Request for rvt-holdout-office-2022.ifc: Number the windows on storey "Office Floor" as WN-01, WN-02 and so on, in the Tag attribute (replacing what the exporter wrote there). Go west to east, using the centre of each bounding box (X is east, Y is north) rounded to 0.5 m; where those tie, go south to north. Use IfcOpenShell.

First a look at what the model holds.

```python
import ifcopenshell
import ifcopenshell.util.element
import ifcopenshell.util.placement

model = ifcopenshell.open("rvt-holdout-office-2022.ifc")
print(model.schema)
storey = next(s for s in model.by_type("IfcBuildingStorey") if s.Name == "Office Floor")
windows = [e for e in ifcopenshell.util.element.get_decomposition(storey) if e.is_a("IfcWindow")]
for e in sorted(windows, key=lambda e: e.id()):
    origin = ifcopenshell.util.placement.get_local_placement(e.ObjectPlacement)[:3, 3]
    print(e.id(), e.Tag, e.Name, origin.round(2) + 0.0, sep=" | ")
```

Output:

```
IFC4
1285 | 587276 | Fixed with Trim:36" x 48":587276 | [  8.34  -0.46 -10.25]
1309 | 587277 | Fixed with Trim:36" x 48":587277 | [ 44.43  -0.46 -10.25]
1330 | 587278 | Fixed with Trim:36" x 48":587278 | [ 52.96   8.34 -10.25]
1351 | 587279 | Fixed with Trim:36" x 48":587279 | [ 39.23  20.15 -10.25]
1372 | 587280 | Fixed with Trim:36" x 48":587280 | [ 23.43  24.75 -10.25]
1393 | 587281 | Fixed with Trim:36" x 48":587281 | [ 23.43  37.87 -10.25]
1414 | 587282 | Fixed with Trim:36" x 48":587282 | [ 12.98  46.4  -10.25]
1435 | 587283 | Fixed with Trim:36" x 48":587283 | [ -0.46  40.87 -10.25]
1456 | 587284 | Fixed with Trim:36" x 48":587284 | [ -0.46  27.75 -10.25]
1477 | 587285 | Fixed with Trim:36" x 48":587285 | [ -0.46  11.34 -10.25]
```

```python
import ifcopenshell
import ifcopenshell.geom
import ifcopenshell.util.element
import ifcopenshell.util.shape

model = ifcopenshell.open("rvt-holdout-office-2022.ifc")
settings = ifcopenshell.geom.settings()
settings.set("use-world-coords", True)


def centre(element):
    shape = ifcopenshell.geom.create_shape(settings, element)
    return ifcopenshell.util.shape.get_bbox_centroid(shape.geometry)


storey = next(s for s in model.by_type("IfcBuildingStorey") if s.Name == "Office Floor")
windows = [e for e in ifcopenshell.util.element.get_decomposition(storey) if e.is_a("IfcWindow")]

# Insertion points can sit at a corner or the storey origin, so sort by the geometry (in metres).
centres = {e: centre(e) for e in windows}
windows.sort(key=lambda e: (round(centres[e][0] / 0.5), centres[e][1]))

for i, e in enumerate(windows, start=1):
    number = f"WN-{i:02d}"
    e.Tag = number
    print(e.id(), number)

model.write("rvt-holdout-office-2022_edited.ifc")
```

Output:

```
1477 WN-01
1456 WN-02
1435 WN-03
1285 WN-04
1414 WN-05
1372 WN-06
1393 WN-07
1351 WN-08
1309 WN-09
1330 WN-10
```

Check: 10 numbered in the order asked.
